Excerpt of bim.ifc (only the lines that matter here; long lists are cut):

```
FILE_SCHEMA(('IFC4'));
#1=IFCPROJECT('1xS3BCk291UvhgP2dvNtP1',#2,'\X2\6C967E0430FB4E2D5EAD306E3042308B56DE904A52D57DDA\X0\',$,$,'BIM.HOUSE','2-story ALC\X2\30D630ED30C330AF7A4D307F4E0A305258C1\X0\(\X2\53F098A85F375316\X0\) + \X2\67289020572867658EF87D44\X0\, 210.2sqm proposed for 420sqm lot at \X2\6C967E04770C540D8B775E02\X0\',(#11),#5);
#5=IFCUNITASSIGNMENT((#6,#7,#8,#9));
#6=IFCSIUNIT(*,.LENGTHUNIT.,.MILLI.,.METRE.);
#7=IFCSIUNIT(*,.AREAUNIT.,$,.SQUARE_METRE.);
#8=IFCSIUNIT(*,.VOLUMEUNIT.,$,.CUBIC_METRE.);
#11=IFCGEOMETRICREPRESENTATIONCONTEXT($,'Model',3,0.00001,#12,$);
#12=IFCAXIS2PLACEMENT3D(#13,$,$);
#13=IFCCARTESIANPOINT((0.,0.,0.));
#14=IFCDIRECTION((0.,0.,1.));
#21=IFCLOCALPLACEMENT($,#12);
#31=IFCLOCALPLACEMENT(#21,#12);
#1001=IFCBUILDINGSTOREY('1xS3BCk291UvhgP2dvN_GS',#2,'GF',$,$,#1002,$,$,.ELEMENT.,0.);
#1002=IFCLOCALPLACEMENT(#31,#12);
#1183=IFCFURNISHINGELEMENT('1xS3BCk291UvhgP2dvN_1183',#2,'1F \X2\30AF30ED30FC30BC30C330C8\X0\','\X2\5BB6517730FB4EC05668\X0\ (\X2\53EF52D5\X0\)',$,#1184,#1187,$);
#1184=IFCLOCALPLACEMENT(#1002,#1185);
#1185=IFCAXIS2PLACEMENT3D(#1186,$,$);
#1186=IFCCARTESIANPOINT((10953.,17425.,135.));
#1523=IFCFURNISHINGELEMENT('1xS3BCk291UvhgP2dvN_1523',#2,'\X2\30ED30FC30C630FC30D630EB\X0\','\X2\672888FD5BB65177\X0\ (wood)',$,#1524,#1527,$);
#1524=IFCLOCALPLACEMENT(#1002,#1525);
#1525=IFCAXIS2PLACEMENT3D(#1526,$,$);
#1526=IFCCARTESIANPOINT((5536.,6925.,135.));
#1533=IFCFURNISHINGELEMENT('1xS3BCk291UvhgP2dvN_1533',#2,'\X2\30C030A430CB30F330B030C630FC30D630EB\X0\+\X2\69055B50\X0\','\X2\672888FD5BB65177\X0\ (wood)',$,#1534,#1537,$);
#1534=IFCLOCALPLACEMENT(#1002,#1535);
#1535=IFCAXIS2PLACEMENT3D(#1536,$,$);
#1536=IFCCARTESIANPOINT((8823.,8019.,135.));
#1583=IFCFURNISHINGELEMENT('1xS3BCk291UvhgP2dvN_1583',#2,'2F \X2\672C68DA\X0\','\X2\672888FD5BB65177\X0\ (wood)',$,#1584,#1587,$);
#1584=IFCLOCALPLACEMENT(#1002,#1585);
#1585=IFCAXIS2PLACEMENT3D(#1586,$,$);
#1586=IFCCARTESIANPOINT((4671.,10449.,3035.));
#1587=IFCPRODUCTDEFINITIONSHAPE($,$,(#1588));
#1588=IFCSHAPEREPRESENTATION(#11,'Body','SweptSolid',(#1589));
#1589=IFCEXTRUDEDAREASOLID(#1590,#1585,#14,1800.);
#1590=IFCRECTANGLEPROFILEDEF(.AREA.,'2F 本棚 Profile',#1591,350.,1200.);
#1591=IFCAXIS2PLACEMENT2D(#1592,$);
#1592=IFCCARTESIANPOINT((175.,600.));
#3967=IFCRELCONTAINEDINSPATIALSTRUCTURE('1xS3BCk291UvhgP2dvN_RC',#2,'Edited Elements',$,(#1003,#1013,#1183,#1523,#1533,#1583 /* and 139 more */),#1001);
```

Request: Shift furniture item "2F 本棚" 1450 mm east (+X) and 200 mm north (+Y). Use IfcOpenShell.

```python
import ifcopenshell
import ifcopenshell.api.geometry
import ifcopenshell.util.placement

model = ifcopenshell.open("bim.ifc")

item = model.by_guid("1xS3BCk291UvhgP2dvN_1583")
matrix = ifcopenshell.util.placement.get_local_placement(item.ObjectPlacement)
matrix[0, 3] += 1450.0
matrix[1, 3] += 200.0
ifcopenshell.api.geometry.edit_object_placement(model, product=item, matrix=matrix, is_si=False)

print(ifcopenshell.util.placement.get_local_placement(item.ObjectPlacement).round(3) + 0.0)

model.write("bim_v2.ifc")
```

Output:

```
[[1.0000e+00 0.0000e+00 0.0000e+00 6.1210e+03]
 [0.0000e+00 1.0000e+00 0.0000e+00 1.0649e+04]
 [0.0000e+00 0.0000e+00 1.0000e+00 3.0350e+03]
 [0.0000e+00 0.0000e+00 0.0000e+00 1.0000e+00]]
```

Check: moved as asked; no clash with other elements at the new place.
